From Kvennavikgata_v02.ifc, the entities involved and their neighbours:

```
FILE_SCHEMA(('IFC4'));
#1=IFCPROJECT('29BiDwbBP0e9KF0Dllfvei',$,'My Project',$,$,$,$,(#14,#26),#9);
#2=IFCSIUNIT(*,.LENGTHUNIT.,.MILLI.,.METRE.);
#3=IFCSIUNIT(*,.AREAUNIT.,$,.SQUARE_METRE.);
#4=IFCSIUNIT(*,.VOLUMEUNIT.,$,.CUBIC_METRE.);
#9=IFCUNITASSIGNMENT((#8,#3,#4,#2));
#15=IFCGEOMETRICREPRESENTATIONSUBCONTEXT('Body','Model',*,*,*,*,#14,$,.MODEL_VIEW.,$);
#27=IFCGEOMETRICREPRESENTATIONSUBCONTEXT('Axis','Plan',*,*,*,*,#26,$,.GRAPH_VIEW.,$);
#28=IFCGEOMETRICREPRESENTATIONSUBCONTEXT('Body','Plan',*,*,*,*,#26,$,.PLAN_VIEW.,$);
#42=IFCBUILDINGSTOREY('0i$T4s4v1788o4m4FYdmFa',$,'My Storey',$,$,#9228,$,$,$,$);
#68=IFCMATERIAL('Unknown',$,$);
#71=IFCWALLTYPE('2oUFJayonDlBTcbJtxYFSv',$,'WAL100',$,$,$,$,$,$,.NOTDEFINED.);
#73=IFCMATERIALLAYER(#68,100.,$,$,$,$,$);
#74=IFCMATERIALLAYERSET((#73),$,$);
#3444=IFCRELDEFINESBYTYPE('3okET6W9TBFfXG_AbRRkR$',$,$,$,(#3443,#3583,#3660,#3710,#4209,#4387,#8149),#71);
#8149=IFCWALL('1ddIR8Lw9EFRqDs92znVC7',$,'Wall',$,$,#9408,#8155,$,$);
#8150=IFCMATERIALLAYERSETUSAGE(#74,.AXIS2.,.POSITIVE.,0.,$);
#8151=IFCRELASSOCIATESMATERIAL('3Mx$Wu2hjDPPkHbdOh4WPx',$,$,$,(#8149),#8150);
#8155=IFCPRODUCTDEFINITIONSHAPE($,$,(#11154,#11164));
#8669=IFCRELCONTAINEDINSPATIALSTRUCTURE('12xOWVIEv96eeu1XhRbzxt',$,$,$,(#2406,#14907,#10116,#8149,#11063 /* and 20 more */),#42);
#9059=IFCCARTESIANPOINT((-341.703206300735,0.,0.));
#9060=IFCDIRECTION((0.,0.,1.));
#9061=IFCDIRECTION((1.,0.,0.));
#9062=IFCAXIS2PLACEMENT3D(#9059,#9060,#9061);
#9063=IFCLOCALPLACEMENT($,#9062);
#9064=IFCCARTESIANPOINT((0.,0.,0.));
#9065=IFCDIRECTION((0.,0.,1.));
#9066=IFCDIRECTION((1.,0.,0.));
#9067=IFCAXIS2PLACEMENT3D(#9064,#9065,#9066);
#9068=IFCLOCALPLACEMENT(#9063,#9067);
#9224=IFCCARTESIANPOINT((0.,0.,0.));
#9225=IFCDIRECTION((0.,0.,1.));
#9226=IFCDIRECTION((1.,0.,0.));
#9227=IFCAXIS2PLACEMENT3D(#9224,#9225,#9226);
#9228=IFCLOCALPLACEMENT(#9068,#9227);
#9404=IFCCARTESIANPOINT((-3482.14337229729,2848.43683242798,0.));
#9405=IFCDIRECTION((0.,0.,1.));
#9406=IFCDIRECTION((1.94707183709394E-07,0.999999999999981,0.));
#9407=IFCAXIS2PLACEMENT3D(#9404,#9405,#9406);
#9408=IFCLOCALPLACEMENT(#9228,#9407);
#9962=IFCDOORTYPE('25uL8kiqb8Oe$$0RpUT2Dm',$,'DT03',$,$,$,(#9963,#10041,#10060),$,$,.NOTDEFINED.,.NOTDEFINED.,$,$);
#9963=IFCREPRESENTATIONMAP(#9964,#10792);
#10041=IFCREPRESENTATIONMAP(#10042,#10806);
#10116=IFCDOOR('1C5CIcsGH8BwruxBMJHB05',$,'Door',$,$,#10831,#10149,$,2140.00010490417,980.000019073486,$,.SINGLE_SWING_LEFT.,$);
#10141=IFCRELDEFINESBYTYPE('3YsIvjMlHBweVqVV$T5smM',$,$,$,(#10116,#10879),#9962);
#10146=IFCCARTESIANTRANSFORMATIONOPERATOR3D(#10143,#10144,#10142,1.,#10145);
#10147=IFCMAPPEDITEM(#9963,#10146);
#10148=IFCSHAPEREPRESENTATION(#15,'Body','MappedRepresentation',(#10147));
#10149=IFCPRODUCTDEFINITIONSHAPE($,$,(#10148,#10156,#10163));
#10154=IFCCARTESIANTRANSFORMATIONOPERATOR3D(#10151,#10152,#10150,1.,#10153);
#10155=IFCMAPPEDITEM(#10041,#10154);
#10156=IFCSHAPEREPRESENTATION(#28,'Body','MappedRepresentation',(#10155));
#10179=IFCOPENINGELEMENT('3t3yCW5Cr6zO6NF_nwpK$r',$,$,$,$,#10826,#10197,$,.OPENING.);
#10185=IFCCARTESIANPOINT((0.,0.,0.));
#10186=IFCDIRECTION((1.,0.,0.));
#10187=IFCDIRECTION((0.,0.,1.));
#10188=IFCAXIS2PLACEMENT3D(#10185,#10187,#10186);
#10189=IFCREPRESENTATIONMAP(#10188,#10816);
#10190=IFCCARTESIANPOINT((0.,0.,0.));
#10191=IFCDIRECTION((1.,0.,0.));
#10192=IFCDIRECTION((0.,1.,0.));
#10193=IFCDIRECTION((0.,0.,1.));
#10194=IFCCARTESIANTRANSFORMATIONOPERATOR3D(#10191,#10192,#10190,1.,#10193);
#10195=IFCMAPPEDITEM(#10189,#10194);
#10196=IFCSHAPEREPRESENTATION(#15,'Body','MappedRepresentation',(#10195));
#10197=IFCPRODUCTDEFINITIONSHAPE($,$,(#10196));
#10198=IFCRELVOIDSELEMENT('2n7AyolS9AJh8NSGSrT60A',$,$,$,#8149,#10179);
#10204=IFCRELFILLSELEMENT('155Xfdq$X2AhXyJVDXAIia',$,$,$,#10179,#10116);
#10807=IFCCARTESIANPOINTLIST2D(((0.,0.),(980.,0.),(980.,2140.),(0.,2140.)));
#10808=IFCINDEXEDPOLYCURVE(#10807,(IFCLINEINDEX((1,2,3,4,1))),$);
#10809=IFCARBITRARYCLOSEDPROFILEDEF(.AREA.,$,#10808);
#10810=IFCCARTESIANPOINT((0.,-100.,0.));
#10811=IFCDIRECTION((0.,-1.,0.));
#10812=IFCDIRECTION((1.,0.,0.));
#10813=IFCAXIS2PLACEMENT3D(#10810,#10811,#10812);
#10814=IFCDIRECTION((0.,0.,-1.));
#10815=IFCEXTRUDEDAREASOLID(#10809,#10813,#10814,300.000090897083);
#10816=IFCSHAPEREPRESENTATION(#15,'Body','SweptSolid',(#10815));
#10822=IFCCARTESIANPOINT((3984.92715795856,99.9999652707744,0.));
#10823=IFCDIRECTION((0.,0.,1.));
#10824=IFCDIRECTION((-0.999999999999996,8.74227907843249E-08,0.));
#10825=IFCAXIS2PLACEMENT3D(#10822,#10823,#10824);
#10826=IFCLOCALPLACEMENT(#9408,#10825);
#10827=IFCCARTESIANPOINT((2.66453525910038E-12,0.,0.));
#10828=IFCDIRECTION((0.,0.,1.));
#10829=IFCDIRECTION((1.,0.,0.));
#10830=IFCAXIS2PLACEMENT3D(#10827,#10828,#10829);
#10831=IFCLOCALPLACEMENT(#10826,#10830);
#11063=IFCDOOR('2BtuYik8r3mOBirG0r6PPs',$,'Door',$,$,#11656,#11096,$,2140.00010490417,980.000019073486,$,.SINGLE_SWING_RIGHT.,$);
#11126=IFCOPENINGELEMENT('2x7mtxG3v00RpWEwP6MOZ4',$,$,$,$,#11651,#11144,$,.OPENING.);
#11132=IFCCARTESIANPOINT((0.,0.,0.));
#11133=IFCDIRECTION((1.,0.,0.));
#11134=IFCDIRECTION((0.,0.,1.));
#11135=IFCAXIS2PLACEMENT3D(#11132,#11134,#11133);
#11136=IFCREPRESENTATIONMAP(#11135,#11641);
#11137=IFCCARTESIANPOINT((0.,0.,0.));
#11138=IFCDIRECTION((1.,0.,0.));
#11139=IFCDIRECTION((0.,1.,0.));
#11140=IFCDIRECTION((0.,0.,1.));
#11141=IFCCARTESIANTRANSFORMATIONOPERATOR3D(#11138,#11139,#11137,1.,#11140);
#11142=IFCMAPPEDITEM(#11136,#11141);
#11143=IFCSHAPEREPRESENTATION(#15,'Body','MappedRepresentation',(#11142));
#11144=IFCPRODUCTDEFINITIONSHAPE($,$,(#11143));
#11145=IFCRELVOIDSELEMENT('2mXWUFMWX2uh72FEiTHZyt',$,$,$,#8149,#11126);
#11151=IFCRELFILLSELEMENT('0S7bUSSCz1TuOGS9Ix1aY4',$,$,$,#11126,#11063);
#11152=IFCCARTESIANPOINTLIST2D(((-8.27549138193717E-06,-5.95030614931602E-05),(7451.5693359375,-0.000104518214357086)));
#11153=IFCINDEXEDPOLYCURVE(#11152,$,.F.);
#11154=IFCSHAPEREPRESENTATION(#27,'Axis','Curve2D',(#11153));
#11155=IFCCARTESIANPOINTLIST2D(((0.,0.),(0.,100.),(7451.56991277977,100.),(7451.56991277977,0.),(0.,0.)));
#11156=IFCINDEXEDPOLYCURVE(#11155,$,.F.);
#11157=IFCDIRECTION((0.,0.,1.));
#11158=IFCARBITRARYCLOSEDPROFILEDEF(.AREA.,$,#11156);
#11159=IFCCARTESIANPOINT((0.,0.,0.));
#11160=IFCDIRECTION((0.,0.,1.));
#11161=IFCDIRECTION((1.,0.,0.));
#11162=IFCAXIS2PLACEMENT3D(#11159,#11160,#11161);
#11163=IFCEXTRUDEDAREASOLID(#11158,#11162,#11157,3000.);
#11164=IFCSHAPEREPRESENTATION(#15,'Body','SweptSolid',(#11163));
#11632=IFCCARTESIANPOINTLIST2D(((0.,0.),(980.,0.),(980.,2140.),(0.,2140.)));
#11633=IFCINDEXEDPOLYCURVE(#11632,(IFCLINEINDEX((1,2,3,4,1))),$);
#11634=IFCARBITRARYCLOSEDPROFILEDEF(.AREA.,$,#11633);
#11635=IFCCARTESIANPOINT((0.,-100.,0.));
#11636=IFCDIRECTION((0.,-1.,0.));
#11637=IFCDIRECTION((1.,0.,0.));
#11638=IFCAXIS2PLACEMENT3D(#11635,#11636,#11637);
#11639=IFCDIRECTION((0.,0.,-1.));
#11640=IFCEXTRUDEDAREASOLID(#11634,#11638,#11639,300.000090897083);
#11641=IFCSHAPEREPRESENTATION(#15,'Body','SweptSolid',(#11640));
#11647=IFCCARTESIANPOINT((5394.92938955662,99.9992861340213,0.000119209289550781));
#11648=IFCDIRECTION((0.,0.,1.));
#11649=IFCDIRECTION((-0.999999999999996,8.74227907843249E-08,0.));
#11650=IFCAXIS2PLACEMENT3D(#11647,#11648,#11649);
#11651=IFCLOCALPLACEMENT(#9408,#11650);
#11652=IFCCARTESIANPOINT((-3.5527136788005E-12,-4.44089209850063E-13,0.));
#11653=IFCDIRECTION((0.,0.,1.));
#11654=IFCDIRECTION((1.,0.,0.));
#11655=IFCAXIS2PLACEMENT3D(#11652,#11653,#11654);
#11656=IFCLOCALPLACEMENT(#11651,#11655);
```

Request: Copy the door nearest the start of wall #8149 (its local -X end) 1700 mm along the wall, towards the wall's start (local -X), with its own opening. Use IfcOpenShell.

```python
import ifcopenshell
import ifcopenshell.api.feature
import ifcopenshell.api.geometry
import ifcopenshell.api.root
import ifcopenshell.geom
import ifcopenshell.util.element
import ifcopenshell.util.placement
import ifcopenshell.util.shape

model = ifcopenshell.open("Kvennavikgata_v02.ifc")
settings = ifcopenshell.geom.settings()


def volume(element):
    """Net volume in cubic metres, openings subtracted."""
    shape = ifcopenshell.geom.create_shape(settings, element)
    return ifcopenshell.util.shape.get_volume(shape.geometry)


door = model.by_guid("1C5CIcsGH8BwruxBMJHB05")
opening = door.FillsVoids[0].RelatingOpeningElement
wall = opening.VoidsElements[0].RelatingBuildingElement
before = volume(wall)
shift = ifcopenshell.util.placement.get_local_placement(wall.ObjectPlacement)[:3, 0] * -1700.0

# copy_class copies the void relationship, type, container and properties, but no geometry.
new_opening = ifcopenshell.api.root.copy_class(model, product=opening)
new_opening.Representation = ifcopenshell.util.element.copy_deep(
    model, opening.Representation, exclude=["IfcGeometricRepresentationContext", "IfcRepresentationMap"]
)
new_door = ifcopenshell.api.root.copy_class(model, product=door)
new_door.Representation = ifcopenshell.util.element.copy_deep(
    model, door.Representation, exclude=["IfcGeometricRepresentationContext", "IfcRepresentationMap"]
)
ifcopenshell.api.feature.add_filling(model, opening=new_opening, element=new_door)

for old, new in ((opening, new_opening), (door, new_door)):
    matrix = ifcopenshell.util.placement.get_local_placement(old.ObjectPlacement)
    matrix[:3, 3] += shift
    ifcopenshell.api.geometry.edit_object_placement(model, product=new, matrix=matrix, is_si=False)

after = volume(wall)

print(f"wall volume {before:.3f} -> {after:.3f} m3")

model.write("Kvennavikgata_v02_updated.ifc")
```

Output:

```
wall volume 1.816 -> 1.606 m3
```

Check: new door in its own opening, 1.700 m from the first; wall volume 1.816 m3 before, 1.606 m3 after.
